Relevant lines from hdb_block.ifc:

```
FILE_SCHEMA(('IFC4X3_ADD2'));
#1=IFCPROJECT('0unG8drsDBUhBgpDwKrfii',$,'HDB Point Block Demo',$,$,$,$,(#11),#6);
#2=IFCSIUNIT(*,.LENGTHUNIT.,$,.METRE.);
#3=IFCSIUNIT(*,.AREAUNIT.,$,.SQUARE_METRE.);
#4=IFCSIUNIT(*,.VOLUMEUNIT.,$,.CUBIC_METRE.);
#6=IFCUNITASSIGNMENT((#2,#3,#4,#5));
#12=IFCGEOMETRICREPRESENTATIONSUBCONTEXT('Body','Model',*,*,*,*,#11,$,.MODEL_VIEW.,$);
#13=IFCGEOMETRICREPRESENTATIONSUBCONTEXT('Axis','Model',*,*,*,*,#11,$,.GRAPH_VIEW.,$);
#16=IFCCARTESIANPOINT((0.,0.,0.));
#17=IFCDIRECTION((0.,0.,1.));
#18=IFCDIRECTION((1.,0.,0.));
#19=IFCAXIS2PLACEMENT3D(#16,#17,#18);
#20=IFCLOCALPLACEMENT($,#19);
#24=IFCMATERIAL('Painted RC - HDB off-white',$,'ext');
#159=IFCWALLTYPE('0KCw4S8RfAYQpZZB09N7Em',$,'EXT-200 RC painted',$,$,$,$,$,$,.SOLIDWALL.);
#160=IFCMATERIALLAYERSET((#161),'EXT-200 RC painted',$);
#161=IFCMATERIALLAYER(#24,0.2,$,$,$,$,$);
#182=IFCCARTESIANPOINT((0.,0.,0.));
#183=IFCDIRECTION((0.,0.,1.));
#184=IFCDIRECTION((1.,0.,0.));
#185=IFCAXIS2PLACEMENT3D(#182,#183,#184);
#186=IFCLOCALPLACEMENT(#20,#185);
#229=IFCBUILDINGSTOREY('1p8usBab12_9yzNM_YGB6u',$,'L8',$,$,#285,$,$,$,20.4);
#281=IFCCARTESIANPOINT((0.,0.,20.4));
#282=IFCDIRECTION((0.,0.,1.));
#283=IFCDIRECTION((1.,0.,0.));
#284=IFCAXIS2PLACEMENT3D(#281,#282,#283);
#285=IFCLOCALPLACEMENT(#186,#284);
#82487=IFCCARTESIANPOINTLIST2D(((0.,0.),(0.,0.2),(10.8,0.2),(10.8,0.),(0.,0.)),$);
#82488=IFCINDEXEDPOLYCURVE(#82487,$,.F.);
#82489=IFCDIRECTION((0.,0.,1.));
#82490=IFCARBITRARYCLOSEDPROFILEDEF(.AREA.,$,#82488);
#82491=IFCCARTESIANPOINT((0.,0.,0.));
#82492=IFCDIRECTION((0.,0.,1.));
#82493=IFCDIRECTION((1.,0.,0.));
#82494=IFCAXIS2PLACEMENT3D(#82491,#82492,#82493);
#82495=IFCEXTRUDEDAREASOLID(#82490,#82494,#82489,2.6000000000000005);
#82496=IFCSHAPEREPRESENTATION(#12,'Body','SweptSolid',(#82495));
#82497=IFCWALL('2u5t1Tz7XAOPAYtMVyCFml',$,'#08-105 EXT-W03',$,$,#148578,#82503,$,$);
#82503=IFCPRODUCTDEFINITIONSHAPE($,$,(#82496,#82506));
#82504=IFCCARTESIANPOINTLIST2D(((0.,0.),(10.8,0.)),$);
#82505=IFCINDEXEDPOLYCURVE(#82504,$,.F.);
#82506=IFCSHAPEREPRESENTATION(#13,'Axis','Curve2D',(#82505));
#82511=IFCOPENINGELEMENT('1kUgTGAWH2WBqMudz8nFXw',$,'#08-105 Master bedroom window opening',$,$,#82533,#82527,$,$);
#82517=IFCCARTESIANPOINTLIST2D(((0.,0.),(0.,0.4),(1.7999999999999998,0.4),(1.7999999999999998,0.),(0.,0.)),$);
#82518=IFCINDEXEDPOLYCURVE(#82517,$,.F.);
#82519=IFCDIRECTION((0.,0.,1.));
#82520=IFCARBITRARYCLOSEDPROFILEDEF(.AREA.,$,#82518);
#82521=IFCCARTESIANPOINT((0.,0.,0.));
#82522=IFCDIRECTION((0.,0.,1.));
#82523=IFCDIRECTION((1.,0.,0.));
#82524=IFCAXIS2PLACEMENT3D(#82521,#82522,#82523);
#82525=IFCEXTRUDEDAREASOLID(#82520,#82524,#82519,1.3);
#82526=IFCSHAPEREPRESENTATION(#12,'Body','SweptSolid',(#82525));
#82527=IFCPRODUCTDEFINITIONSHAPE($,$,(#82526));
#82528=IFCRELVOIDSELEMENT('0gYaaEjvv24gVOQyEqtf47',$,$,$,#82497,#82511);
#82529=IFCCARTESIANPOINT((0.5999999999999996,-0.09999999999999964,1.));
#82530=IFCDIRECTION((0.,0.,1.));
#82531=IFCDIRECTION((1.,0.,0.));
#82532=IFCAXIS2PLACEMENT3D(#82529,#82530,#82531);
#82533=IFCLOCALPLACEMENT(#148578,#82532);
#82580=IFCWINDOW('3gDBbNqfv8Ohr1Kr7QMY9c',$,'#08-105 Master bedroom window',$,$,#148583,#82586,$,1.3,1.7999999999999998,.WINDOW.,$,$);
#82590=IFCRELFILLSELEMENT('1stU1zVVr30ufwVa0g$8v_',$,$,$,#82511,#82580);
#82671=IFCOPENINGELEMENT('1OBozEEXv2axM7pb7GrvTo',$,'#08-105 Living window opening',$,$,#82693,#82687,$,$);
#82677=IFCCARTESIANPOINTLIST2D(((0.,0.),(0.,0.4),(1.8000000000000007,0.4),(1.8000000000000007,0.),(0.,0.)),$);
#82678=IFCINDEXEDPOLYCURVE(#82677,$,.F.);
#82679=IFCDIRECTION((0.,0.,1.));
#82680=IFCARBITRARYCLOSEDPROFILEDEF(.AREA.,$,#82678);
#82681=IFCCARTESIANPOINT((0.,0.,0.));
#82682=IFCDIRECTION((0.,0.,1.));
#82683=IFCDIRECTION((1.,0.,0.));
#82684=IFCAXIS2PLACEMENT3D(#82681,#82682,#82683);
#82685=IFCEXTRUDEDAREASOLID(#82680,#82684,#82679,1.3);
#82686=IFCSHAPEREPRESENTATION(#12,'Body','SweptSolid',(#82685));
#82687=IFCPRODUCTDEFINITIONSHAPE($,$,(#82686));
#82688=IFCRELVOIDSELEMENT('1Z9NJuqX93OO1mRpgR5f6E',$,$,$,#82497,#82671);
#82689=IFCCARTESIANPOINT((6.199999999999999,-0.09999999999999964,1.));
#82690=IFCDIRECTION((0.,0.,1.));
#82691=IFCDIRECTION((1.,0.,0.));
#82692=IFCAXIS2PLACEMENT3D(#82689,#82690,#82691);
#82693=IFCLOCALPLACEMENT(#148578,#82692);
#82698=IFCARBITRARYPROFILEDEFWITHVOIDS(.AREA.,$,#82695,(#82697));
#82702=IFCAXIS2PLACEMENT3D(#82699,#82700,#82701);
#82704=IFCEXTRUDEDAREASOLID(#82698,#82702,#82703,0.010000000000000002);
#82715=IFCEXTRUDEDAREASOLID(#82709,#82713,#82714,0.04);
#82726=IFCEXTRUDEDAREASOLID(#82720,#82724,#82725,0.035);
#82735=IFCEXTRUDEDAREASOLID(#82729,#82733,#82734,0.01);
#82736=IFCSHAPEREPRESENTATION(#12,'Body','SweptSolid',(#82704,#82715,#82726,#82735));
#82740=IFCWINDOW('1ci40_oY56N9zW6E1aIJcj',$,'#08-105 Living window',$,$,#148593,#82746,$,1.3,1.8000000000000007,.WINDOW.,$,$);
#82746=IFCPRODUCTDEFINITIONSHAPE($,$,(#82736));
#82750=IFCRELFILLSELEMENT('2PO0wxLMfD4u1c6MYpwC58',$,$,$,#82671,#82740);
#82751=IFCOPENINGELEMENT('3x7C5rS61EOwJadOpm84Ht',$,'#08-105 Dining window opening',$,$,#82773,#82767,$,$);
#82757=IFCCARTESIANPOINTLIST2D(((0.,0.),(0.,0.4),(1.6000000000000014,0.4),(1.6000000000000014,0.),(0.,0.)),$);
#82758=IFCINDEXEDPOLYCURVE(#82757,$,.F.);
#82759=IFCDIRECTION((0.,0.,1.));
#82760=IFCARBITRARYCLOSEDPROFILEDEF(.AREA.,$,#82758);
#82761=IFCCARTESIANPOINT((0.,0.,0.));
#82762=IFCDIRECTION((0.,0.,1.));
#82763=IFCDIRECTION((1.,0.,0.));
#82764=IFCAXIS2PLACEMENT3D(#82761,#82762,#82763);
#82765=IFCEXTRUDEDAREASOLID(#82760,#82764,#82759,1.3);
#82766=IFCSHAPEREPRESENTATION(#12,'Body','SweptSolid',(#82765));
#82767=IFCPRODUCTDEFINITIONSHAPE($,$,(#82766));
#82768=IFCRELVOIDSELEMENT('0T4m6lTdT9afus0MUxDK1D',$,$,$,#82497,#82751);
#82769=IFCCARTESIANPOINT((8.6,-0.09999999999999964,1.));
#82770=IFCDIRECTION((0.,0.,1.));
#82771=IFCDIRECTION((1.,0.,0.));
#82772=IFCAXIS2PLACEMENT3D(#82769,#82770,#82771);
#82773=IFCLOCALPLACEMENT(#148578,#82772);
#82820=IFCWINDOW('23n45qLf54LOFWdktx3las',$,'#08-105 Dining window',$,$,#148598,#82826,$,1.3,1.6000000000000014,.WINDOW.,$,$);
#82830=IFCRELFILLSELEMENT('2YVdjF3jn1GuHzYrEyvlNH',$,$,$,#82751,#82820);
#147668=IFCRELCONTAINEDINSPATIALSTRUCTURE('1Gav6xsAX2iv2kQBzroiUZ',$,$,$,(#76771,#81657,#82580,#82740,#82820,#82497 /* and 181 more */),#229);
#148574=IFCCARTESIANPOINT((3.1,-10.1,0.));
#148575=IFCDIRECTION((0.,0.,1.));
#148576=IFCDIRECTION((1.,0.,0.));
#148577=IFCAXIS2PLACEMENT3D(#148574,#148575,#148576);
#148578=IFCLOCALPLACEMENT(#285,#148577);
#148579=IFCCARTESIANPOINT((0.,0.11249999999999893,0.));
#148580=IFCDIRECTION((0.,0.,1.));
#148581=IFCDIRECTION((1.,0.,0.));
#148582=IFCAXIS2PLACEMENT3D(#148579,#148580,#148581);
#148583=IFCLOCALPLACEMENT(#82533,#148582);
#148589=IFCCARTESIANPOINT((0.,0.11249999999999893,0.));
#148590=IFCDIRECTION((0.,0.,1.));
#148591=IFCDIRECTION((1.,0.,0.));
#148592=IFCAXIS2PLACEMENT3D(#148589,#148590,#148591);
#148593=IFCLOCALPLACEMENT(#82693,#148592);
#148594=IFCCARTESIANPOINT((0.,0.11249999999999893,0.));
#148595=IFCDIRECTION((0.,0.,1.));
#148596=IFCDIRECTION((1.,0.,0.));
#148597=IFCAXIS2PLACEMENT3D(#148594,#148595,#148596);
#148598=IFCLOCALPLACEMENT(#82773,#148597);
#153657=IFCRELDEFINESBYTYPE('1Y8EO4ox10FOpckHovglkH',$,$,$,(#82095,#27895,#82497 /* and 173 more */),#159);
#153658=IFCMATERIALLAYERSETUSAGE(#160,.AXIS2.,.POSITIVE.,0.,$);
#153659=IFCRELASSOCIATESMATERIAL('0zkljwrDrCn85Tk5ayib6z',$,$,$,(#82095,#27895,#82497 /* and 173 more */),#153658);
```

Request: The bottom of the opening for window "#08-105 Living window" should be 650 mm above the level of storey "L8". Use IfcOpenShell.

```python
import numpy as np
import ifcopenshell
import ifcopenshell.api.geometry
import ifcopenshell.geom
import ifcopenshell.util.element
import ifcopenshell.util.placement
import ifcopenshell.util.shape
import ifcopenshell.util.unit

model = ifcopenshell.open("hdb_block.ifc")
unit_scale = ifcopenshell.util.unit.calculate_unit_scale(model)

window = model.by_guid("1ci40_oY56N9zW6E1aIJcj")
opening = window.FillsVoids[0].RelatingOpeningElement
storey = ifcopenshell.util.element.get_container(window, ifc_class="IfcBuildingStorey")
level = ifcopenshell.util.placement.get_local_placement(storey.ObjectPlacement)[2, 3]

# The opening's origin need not be at the sill, so measure its lowest point.
shape = ifcopenshell.geom.create_shape(ifcopenshell.geom.settings(), opening)
bottom = ifcopenshell.util.shape.get_shape_bottom_elevation(shape, shape.geometry) / unit_scale
dz = level + 0.65 / unit_scale - bottom

shift = np.array([0.0, 0.0, dz])
# The window is placed relative to its opening, so it follows when the opening moves.
matrix = ifcopenshell.util.placement.get_local_placement(opening.ObjectPlacement)
matrix[:3, 3] += shift
ifcopenshell.api.geometry.edit_object_placement(
    model, product=opening, matrix=matrix, is_si=False, should_transform_children=True
)

print(f"moved by {dz * unit_scale:+.3f} m")

model.write("hdb_block_rev.ifc")
```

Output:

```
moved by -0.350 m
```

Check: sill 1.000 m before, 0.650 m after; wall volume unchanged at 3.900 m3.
